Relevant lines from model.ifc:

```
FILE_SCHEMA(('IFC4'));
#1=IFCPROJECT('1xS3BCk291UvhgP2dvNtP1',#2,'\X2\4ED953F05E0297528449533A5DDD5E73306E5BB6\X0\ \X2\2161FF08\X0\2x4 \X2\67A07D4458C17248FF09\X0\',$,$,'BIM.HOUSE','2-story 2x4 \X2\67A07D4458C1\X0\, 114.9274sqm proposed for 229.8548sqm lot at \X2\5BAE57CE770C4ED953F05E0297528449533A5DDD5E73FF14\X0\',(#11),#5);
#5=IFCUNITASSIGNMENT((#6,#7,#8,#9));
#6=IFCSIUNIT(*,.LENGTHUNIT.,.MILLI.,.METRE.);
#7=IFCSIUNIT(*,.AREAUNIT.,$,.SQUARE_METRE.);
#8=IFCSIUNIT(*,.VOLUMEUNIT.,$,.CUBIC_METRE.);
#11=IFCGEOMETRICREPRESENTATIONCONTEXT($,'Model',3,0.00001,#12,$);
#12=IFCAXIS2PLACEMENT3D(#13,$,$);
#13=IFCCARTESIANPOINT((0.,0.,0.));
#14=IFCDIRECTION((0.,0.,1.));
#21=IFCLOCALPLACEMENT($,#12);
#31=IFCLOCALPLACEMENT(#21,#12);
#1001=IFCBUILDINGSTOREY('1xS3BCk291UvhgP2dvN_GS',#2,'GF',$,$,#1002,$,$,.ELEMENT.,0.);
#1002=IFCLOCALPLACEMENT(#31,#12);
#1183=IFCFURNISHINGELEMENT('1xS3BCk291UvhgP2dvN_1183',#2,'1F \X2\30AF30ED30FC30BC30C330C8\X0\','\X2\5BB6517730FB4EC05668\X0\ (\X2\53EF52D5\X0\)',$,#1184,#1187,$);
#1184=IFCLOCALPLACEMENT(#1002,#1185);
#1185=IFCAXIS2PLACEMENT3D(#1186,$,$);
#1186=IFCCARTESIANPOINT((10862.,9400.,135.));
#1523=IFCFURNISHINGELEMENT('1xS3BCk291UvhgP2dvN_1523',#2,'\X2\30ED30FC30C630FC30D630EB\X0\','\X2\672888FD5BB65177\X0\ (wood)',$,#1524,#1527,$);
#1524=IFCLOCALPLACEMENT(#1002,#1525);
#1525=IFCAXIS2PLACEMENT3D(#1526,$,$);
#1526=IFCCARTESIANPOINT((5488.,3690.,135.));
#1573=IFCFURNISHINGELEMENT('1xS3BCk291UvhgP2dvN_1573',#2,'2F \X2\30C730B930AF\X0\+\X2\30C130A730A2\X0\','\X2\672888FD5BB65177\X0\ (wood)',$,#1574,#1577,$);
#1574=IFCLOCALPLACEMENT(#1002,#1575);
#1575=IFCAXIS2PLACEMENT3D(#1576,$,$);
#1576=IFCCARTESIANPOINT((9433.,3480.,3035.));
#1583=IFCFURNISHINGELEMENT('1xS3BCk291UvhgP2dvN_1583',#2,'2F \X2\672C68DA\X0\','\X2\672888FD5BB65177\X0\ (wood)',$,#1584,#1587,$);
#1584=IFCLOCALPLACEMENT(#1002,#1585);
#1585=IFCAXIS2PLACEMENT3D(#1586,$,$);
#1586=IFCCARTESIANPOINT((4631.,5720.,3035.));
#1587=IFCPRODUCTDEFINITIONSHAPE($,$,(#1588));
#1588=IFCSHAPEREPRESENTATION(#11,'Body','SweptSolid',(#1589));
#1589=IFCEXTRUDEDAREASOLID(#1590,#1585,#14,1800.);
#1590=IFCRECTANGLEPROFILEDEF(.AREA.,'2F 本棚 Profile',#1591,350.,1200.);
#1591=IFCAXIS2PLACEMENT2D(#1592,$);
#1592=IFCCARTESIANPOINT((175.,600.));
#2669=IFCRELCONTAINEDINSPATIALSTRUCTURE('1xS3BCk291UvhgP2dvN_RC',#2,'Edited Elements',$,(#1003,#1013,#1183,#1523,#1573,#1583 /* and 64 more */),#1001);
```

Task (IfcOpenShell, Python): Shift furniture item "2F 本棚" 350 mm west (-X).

```python
import ifcopenshell
import ifcopenshell.api.geometry
import ifcopenshell.util.placement
import ifcopenshell.util.unit

model = ifcopenshell.open("model.ifc")
unit_scale = ifcopenshell.util.unit.calculate_unit_scale(model)

item = model.by_guid("1xS3BCk291UvhgP2dvN_1583")
matrix = ifcopenshell.util.placement.get_local_placement(item.ObjectPlacement)
matrix[0, 3] -= 0.35 / unit_scale
ifcopenshell.api.geometry.edit_object_placement(model, product=item, matrix=matrix, is_si=False)

print(ifcopenshell.util.placement.get_local_placement(item.ObjectPlacement).round(3) + 0.0)

model.write("model_rev.ifc")
```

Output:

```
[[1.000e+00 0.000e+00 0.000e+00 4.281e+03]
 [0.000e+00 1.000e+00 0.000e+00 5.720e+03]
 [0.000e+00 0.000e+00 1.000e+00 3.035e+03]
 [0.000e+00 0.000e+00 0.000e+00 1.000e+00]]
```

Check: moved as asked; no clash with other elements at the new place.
